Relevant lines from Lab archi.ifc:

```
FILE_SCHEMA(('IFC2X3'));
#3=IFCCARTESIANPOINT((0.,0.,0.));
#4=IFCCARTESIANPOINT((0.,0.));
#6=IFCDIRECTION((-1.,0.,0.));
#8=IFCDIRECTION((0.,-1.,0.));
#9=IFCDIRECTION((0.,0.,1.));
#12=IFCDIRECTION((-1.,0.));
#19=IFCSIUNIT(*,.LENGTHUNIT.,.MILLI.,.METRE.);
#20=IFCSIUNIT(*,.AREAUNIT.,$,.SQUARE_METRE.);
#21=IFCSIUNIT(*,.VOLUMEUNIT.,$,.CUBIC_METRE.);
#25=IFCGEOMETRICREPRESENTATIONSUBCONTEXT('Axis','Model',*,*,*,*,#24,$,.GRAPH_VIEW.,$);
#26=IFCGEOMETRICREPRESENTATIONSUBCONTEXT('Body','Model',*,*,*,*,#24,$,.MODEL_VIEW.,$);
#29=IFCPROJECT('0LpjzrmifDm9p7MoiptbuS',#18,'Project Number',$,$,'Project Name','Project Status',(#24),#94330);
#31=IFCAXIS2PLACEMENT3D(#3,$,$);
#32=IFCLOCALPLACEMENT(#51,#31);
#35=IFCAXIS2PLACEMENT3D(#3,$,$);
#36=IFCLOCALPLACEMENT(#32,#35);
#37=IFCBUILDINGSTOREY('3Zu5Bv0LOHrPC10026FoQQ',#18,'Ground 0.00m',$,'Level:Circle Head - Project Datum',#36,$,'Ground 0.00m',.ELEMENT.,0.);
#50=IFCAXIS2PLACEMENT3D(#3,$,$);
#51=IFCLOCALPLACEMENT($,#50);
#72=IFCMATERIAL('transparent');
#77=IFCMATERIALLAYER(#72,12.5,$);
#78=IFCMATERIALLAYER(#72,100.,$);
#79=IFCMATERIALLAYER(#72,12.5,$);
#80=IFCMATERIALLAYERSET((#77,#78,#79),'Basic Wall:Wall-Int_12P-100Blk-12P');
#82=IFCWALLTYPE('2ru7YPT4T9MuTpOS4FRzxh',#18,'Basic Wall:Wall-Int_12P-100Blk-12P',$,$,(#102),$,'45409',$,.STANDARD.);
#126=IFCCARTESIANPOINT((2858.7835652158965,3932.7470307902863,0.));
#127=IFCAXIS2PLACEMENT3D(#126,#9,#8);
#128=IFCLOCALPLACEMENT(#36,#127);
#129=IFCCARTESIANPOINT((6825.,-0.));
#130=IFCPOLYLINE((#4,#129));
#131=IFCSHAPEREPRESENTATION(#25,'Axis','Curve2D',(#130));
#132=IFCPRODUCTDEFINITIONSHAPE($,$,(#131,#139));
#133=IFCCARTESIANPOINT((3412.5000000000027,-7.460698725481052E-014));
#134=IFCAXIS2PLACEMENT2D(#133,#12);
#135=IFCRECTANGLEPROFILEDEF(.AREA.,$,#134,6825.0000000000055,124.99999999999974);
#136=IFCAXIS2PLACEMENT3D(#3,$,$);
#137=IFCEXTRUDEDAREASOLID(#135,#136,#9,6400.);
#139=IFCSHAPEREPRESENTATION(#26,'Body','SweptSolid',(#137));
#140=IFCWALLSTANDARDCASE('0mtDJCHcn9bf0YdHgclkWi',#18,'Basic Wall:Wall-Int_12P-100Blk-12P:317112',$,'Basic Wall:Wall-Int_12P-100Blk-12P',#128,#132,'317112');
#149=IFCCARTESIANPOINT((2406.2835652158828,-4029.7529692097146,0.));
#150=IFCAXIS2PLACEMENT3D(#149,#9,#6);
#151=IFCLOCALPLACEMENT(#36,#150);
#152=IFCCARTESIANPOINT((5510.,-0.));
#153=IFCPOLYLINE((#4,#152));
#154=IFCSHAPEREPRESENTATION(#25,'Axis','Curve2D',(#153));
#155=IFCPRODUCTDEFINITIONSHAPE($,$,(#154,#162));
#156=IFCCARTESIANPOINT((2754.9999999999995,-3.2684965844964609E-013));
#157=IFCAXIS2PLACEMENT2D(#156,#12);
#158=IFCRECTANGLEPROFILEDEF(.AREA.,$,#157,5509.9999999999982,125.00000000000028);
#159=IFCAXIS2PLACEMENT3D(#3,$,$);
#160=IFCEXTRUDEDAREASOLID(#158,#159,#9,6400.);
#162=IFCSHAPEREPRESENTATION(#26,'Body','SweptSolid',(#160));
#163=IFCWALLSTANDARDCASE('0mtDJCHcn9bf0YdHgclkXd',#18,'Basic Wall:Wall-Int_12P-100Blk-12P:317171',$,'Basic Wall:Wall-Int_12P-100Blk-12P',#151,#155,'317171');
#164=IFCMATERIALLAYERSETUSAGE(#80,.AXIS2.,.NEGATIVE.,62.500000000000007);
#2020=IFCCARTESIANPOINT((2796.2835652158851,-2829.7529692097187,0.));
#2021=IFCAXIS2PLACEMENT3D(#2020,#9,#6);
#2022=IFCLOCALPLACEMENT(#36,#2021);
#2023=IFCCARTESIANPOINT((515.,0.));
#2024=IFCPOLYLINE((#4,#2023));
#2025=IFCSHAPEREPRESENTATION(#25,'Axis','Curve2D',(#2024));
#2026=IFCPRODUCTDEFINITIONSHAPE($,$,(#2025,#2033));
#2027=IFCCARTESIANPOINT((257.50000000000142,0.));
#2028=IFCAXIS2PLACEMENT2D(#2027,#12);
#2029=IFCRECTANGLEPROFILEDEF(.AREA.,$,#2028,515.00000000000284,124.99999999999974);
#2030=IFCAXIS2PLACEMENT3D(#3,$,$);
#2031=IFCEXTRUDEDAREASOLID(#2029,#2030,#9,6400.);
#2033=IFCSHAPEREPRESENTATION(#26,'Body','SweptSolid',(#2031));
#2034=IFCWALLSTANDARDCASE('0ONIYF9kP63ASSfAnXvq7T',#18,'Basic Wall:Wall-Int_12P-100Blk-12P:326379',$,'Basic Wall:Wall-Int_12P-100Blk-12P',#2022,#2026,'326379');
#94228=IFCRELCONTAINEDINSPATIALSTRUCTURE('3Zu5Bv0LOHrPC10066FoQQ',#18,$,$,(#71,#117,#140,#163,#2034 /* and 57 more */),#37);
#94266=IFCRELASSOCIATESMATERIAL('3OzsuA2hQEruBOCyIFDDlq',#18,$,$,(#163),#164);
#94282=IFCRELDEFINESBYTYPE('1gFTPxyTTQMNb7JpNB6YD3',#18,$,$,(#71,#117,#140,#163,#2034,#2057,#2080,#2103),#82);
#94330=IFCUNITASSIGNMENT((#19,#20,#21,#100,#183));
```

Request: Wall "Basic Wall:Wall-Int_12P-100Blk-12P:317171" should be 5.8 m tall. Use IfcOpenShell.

```python
import ifcopenshell
import ifcopenshell.geom
import ifcopenshell.util.representation
import ifcopenshell.util.shape
import ifcopenshell.util.unit

model = ifcopenshell.open("Lab archi.ifc")
unit_scale = ifcopenshell.util.unit.calculate_unit_scale(model)
settings = ifcopenshell.geom.settings()


def volume(element):
    """Net volume in cubic metres, openings subtracted."""
    shape = ifcopenshell.geom.create_shape(settings, element)
    return ifcopenshell.util.shape.get_volume(shape.geometry)


wall = model.by_id(163)
before = volume(wall)

body = ifcopenshell.util.representation.get_representation(wall, "Model", "Body")
solid = body.Items[0]
old_height = solid.Depth
solid.Depth = 5.8 / unit_scale
after = volume(wall)

print(f"height {old_height:g} -> {solid.Depth:g}, volume {before:.3f} -> {after:.3f} m3")

model.write("Lab archi_updated.ifc")
```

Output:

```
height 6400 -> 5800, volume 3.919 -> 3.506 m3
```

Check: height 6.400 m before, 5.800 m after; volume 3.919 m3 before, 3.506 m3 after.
